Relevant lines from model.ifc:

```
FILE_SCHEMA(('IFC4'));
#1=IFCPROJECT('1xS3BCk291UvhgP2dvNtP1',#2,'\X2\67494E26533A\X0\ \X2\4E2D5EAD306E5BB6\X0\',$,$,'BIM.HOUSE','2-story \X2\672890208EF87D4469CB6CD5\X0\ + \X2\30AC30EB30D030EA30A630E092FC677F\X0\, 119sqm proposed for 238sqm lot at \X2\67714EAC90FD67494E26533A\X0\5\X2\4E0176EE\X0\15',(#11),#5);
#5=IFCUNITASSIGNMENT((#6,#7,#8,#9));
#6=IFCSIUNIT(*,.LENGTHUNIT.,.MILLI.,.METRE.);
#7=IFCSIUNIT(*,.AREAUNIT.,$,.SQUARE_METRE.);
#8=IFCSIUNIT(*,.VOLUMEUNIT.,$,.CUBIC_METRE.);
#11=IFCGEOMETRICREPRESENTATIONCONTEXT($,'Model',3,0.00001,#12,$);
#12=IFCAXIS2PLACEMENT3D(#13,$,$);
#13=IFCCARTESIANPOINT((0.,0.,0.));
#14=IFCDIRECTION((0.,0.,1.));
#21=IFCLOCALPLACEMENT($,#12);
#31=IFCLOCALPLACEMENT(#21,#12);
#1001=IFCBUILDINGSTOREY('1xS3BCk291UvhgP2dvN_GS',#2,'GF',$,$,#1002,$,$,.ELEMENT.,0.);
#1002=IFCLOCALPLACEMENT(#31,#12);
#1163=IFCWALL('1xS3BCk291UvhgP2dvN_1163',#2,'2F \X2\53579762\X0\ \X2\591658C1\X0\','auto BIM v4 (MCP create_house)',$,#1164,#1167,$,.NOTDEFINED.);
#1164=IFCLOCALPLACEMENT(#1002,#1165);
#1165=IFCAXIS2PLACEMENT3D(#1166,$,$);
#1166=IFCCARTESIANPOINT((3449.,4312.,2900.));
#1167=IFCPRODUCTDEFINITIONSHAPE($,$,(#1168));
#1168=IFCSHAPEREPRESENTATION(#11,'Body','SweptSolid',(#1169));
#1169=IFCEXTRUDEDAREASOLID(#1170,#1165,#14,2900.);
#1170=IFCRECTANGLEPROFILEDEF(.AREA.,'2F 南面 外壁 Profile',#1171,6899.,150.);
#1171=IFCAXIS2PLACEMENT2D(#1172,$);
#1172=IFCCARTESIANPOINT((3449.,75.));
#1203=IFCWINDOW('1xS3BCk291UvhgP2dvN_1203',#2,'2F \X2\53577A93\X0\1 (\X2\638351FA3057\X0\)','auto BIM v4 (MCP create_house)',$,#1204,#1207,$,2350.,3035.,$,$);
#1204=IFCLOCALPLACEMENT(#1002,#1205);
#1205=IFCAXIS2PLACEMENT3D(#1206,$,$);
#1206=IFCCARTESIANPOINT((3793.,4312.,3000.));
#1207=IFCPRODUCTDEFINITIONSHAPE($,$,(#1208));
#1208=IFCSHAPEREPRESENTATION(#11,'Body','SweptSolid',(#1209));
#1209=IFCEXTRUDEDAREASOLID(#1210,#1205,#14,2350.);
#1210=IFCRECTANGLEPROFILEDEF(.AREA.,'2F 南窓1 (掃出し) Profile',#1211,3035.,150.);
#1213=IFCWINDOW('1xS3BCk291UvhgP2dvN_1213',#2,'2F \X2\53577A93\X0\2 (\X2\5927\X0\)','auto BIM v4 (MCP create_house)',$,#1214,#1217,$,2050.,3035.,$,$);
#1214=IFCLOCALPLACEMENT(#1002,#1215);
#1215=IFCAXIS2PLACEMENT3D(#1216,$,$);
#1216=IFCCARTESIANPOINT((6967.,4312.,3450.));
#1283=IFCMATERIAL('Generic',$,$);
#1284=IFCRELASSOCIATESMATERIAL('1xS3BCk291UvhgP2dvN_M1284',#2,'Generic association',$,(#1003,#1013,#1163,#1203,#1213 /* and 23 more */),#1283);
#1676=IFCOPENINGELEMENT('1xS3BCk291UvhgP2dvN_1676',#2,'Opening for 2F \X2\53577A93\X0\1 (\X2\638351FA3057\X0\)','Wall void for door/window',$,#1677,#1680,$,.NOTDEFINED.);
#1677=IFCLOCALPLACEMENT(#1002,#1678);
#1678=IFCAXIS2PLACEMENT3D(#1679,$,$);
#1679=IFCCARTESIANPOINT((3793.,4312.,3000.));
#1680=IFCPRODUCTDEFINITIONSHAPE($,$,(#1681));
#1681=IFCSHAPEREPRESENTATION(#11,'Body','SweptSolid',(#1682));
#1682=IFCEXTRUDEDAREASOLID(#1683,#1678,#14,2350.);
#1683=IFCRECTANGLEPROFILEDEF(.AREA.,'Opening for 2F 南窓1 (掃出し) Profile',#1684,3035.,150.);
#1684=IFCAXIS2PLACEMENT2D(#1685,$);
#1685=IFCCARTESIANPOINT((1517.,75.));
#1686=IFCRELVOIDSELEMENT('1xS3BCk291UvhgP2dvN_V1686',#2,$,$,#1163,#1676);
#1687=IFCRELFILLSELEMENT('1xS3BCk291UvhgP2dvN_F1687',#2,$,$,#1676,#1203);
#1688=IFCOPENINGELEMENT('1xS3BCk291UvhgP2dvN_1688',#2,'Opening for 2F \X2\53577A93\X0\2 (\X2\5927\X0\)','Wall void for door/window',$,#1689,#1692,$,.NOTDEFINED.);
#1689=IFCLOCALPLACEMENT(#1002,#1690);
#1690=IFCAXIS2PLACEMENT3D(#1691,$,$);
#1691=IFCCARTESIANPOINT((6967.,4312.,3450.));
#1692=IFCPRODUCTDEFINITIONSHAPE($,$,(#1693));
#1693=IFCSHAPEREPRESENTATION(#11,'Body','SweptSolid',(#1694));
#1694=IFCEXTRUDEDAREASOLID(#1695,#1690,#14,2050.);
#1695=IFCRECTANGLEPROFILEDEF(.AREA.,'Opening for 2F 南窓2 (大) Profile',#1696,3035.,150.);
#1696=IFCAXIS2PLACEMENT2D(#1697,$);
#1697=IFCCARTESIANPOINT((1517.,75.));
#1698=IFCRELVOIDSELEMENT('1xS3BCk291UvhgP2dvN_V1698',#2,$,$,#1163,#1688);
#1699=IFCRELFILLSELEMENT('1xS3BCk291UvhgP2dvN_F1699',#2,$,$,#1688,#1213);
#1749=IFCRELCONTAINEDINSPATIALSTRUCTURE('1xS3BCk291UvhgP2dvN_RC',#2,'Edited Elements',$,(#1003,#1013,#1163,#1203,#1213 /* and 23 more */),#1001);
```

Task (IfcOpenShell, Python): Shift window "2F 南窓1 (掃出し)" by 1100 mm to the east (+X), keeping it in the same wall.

```python
import ifcopenshell
import ifcopenshell.api.geometry
import ifcopenshell.util.placement
import ifcopenshell.util.unit

model = ifcopenshell.open("model.ifc")
unit_scale = ifcopenshell.util.unit.calculate_unit_scale(model)

window = model.by_guid("1xS3BCk291UvhgP2dvN_1203")
opening = window.FillsVoids[0].RelatingOpeningElement
wall = opening.VoidsElements[0].RelatingBuildingElement

wall_matrix = ifcopenshell.util.placement.get_local_placement(wall.ObjectPlacement)
shift = wall_matrix[:3, 0] * 1.1 / unit_scale
before = ifcopenshell.util.placement.get_local_placement(window.ObjectPlacement)[:3, 3].copy()

# The window is not placed relative to its opening, so move both.
for product in (opening, window):
    matrix = ifcopenshell.util.placement.get_local_placement(product.ObjectPlacement)
    matrix[:3, 3] += shift
    ifcopenshell.api.geometry.edit_object_placement(model, product=product, matrix=matrix, is_si=False)

after = ifcopenshell.util.placement.get_local_placement(window.ObjectPlacement)[:3, 3]
print("window moved by", (after - before).round(3) + 0.0)

model.write("model_edited.ifc")
```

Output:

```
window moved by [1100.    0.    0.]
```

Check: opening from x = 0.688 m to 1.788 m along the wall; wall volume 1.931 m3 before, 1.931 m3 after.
